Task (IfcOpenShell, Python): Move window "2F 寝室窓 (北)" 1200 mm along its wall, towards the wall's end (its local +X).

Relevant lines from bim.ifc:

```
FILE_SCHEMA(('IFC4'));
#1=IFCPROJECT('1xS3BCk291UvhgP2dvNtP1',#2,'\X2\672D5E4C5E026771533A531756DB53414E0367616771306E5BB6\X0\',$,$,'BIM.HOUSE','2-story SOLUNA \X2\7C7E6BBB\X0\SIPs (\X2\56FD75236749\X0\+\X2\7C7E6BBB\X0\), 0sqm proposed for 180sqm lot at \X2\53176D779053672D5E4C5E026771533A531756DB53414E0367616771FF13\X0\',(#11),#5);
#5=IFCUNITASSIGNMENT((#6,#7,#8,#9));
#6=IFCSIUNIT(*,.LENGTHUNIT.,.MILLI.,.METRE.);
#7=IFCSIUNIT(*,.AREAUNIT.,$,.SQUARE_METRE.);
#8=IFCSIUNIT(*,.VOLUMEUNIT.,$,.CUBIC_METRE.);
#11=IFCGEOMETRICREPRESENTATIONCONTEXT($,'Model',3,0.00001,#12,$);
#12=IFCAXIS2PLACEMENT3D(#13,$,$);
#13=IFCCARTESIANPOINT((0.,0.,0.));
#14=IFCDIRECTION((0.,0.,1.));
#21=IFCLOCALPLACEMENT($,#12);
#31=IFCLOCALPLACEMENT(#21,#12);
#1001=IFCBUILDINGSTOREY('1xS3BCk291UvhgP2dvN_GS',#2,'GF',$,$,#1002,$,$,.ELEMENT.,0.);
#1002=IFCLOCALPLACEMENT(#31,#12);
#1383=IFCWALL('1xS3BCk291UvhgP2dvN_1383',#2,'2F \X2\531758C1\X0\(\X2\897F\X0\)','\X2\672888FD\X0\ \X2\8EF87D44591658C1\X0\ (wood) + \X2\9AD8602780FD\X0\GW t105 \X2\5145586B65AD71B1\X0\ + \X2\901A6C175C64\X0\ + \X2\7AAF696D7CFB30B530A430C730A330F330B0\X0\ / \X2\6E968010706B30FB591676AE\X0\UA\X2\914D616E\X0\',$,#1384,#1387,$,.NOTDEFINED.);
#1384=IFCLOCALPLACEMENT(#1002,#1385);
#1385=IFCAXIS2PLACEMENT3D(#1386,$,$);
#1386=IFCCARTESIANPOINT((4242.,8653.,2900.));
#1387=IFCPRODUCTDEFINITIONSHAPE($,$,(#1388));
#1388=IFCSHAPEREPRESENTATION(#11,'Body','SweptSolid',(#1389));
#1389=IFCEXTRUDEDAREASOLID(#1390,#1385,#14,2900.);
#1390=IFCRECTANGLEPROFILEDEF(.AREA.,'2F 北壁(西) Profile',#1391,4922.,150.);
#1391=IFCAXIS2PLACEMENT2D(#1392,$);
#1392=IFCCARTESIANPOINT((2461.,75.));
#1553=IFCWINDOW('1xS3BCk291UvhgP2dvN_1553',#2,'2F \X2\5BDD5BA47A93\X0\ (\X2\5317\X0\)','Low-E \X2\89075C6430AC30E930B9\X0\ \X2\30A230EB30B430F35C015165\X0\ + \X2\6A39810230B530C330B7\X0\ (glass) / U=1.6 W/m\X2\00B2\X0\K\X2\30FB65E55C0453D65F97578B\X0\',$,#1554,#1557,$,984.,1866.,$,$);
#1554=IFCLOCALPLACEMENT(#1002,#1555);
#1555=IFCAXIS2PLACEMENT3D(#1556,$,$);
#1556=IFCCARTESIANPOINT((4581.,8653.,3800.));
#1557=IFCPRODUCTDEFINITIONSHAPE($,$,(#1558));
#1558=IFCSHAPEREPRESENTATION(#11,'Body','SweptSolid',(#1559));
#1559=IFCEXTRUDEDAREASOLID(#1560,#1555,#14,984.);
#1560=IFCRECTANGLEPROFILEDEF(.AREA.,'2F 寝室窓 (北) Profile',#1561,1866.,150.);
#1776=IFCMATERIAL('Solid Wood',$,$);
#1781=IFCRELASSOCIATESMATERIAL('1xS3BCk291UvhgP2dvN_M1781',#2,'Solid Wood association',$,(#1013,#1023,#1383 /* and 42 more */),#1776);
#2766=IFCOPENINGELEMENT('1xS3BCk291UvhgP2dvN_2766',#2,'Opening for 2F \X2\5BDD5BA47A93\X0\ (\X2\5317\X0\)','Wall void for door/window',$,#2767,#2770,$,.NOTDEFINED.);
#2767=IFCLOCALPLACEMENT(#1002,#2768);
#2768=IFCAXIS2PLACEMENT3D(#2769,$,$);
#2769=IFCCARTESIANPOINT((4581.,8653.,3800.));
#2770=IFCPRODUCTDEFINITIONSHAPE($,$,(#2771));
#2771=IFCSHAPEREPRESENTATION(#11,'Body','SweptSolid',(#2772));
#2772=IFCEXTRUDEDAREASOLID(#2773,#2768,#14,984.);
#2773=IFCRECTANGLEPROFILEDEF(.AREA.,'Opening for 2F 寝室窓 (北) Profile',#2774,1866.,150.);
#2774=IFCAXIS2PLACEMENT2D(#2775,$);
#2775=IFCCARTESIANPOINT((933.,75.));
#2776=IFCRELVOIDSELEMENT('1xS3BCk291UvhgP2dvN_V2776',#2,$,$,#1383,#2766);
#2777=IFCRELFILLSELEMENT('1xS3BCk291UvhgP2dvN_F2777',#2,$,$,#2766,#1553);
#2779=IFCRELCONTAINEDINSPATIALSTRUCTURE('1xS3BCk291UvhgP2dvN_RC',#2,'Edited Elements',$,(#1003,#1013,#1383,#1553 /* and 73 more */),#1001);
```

```python
import ifcopenshell
import ifcopenshell.api.geometry
import ifcopenshell.util.placement
import ifcopenshell.util.unit

model = ifcopenshell.open("bim.ifc")
unit_scale = ifcopenshell.util.unit.calculate_unit_scale(model)

window = model.by_id(1553)
opening = window.FillsVoids[0].RelatingOpeningElement
wall = opening.VoidsElements[0].RelatingBuildingElement

wall_matrix = ifcopenshell.util.placement.get_local_placement(wall.ObjectPlacement)
shift = wall_matrix[:3, 0] * 1.2 / unit_scale
before = ifcopenshell.util.placement.get_local_placement(window.ObjectPlacement)[:3, 3].copy()

# The window is not placed relative to its opening, so move both.
for product in (opening, window):
    matrix = ifcopenshell.util.placement.get_local_placement(product.ObjectPlacement)
    matrix[:3, 3] += shift
    ifcopenshell.api.geometry.edit_object_placement(model, product=product, matrix=matrix, is_si=False)

after = ifcopenshell.util.placement.get_local_placement(window.ObjectPlacement)[:3, 3]
print("window moved by", (after - before).round(3) + 0.0)

model.write("bim-out.ifc")
```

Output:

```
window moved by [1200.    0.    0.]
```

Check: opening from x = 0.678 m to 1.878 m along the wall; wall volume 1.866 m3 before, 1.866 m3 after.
